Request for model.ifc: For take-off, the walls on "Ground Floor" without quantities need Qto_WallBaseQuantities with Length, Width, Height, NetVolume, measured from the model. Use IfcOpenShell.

First a look at what the model holds.

```python
import ifcopenshell
import ifcopenshell.util.element
import ifcopenshell.util.unit

model = ifcopenshell.open("model.ifc")
print(model.schema)
for unit_type in ("LENGTHUNIT", "AREAUNIT", "VOLUMEUNIT"):
    print(unit_type, ifcopenshell.util.unit.calculate_unit_scale(model, unit_type))
storey = next(s for s in model.by_type("IfcBuildingStorey") if s.Name == "Ground Floor")
walls = [e for e in ifcopenshell.util.element.get_decomposition(storey) if e.is_a("IfcWall")]
for e in sorted(walls, key=lambda e: e.id()):
    print(e.id(), e.is_a(), e.Name, list(ifcopenshell.util.element.get_psets(e, qtos_only=True)), sep=" | ")
```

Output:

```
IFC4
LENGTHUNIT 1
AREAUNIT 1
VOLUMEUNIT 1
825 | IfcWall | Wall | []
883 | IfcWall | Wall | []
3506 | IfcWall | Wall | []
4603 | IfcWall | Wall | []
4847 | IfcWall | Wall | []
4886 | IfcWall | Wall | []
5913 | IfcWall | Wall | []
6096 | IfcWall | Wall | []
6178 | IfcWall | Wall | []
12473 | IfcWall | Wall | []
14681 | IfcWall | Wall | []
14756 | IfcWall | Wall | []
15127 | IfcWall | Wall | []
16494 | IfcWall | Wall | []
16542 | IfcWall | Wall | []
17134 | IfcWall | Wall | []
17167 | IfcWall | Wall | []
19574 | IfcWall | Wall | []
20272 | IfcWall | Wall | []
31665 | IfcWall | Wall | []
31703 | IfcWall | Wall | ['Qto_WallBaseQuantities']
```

```python
import ifcopenshell
import ifcopenshell.api.pset
import ifcopenshell.geom
import ifcopenshell.util.element
import ifcopenshell.util.shape
import ifcopenshell.util.unit

model = ifcopenshell.open("model.ifc")
unit_scale = ifcopenshell.util.unit.calculate_unit_scale(model)
volume_scale = ifcopenshell.util.unit.calculate_unit_scale(model, "VOLUMEUNIT")
settings = ifcopenshell.geom.settings()

storey = next(s for s in model.by_type("IfcBuildingStorey") if s.Name == "Ground Floor")
walls = [e for e in ifcopenshell.util.element.get_decomposition(storey) if e.is_a("IfcWall")]

for e in sorted(walls, key=lambda e: e.id()):
    if ifcopenshell.util.element.get_psets(e, qtos_only=True, should_inherit=False):
        continue
    # Geometry comes back in metres, in the element's own axes.
    shape = ifcopenshell.geom.create_shape(settings, e)
    values = {
        "Length": ifcopenshell.util.shape.get_x(shape.geometry) / unit_scale,
        "Width": ifcopenshell.util.shape.get_y(shape.geometry) / unit_scale,
        "Height": ifcopenshell.util.shape.get_z(shape.geometry) / unit_scale,
        "NetVolume": ifcopenshell.util.shape.get_volume(shape.geometry) / volume_scale,
    }
    qto = ifcopenshell.api.pset.add_qto(model, product=e, name="Qto_WallBaseQuantities")
    ifcopenshell.api.pset.edit_qto(model, qto=qto, properties=values)
    print(e.id(), {k: round(v, 3) for k, v in values.items()})

model.write("model_updated.ifc")
```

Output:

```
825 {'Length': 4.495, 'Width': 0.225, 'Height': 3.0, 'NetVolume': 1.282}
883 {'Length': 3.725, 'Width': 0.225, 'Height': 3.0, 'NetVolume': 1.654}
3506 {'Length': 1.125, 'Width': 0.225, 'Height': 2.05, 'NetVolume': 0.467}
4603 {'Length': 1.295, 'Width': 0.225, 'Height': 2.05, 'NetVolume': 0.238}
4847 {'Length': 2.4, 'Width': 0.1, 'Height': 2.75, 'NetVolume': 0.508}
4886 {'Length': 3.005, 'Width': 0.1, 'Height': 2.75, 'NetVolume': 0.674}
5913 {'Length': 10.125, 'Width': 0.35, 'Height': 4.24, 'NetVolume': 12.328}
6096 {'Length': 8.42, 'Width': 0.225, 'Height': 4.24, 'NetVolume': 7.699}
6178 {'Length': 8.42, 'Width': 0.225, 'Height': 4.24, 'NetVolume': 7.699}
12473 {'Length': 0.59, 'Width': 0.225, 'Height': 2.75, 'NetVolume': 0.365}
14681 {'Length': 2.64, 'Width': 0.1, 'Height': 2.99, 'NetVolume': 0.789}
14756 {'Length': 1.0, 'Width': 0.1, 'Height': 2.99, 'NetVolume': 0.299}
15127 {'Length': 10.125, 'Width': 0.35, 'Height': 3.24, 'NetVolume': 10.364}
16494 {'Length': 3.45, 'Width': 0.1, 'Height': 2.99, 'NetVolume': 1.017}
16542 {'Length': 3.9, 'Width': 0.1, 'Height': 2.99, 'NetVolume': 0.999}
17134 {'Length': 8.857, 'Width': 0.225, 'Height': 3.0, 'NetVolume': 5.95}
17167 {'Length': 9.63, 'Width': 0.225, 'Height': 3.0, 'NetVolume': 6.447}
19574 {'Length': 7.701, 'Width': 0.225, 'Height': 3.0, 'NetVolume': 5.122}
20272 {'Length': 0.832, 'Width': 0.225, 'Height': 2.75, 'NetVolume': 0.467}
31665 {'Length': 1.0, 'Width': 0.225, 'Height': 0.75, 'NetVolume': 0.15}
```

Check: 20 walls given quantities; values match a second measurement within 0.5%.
